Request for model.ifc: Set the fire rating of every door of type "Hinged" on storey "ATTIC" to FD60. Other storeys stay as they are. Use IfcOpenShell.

First a look at what the model holds.

```python
import ifcopenshell
import ifcopenshell.util.element

model = ifcopenshell.open("model.ifc")
print(model.schema)
storey = next(s for s in model.by_type("IfcBuildingStorey") if s.Name == "ATTIC")
doors = [e for e in ifcopenshell.util.element.get_decomposition(storey) if e.is_a("IfcDoor")]
seen = {}
for e in doors:
    element_type = ifcopenshell.util.element.get_type(e)
    key = (element_type.Name if element_type != e and element_type else None, ifcopenshell.util.element.get_pset(e, "Pset_DoorCommon", "FireRating"))
    seen[key] = seen.get(key, 0) + 1
for (name, value), count in sorted(seen.items(), key=str):
    print(count, "x", name, "|", value)
```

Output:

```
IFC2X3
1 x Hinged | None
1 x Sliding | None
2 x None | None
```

```python
import ifcopenshell
import ifcopenshell.api.pset
import ifcopenshell.util.element

model = ifcopenshell.open("model.ifc")

storey = next(s for s in model.by_type("IfcBuildingStorey") if s.Name == "ATTIC")
doors = [e for e in ifcopenshell.util.element.get_decomposition(storey) if e.is_a("IfcDoor")]

count = 0
for e in doors:
    element_type = ifcopenshell.util.element.get_type(e)
    if element_type in (None, e) or element_type.Name != "Hinged":
        continue
    # add_pset returns the element's existing set when there is one.
    pset = ifcopenshell.api.pset.add_pset(model, product=e, name="Pset_DoorCommon")
    ifcopenshell.api.pset.edit_pset(model, pset=pset, properties={"FireRating": "FD60"})
    count += 1

print(count, "doors updated")

model.write("model_v2.ifc")
```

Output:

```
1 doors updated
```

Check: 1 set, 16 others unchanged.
